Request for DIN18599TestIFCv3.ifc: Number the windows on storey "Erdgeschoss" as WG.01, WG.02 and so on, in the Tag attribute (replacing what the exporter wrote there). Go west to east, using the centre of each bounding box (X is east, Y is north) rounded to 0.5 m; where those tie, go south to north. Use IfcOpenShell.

First a look at what the model holds.

```python
import ifcopenshell
import ifcopenshell.util.element
import ifcopenshell.util.placement

model = ifcopenshell.open("DIN18599TestIFCv3.ifc")
print(model.schema)
storey = next(s for s in model.by_type("IfcBuildingStorey") if s.Name == "Erdgeschoss")
windows = [e for e in ifcopenshell.util.element.get_decomposition(storey) if e.is_a("IfcWindow")]
for e in sorted(windows, key=lambda e: e.id()):
    origin = ifcopenshell.util.placement.get_local_placement(e.ObjectPlacement)[:3, 3]
    print(e.id(), e.Tag, e.Name, origin.round(2) + 0.0, sep=" | ")
```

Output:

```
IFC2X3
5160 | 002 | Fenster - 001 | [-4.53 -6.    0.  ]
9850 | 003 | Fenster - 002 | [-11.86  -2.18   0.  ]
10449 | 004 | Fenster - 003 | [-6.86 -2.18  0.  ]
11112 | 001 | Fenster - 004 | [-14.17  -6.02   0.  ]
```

```python
import ifcopenshell
import ifcopenshell.geom
import ifcopenshell.util.element
import ifcopenshell.util.shape

model = ifcopenshell.open("DIN18599TestIFCv3.ifc")
settings = ifcopenshell.geom.settings()
settings.set("use-world-coords", True)


def centre(element):
    shape = ifcopenshell.geom.create_shape(settings, element)
    return ifcopenshell.util.shape.get_bbox_centroid(shape.geometry)


storey = next(s for s in model.by_type("IfcBuildingStorey") if s.Name == "Erdgeschoss")
windows = [e for e in ifcopenshell.util.element.get_decomposition(storey) if e.is_a("IfcWindow")]

# Insertion points can sit at a corner or the storey origin, so sort by the geometry (in metres).
centres = {e: centre(e) for e in windows}
windows.sort(key=lambda e: (round(centres[e][0] / 0.5), centres[e][1]))

for i, e in enumerate(windows, start=1):
    number = f"WG.{i:02d}"
    e.Tag = number
    print(e.id(), number)

model.write("DIN18599TestIFCv3_v2.ifc")
```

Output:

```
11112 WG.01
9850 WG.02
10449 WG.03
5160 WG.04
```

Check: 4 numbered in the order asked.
